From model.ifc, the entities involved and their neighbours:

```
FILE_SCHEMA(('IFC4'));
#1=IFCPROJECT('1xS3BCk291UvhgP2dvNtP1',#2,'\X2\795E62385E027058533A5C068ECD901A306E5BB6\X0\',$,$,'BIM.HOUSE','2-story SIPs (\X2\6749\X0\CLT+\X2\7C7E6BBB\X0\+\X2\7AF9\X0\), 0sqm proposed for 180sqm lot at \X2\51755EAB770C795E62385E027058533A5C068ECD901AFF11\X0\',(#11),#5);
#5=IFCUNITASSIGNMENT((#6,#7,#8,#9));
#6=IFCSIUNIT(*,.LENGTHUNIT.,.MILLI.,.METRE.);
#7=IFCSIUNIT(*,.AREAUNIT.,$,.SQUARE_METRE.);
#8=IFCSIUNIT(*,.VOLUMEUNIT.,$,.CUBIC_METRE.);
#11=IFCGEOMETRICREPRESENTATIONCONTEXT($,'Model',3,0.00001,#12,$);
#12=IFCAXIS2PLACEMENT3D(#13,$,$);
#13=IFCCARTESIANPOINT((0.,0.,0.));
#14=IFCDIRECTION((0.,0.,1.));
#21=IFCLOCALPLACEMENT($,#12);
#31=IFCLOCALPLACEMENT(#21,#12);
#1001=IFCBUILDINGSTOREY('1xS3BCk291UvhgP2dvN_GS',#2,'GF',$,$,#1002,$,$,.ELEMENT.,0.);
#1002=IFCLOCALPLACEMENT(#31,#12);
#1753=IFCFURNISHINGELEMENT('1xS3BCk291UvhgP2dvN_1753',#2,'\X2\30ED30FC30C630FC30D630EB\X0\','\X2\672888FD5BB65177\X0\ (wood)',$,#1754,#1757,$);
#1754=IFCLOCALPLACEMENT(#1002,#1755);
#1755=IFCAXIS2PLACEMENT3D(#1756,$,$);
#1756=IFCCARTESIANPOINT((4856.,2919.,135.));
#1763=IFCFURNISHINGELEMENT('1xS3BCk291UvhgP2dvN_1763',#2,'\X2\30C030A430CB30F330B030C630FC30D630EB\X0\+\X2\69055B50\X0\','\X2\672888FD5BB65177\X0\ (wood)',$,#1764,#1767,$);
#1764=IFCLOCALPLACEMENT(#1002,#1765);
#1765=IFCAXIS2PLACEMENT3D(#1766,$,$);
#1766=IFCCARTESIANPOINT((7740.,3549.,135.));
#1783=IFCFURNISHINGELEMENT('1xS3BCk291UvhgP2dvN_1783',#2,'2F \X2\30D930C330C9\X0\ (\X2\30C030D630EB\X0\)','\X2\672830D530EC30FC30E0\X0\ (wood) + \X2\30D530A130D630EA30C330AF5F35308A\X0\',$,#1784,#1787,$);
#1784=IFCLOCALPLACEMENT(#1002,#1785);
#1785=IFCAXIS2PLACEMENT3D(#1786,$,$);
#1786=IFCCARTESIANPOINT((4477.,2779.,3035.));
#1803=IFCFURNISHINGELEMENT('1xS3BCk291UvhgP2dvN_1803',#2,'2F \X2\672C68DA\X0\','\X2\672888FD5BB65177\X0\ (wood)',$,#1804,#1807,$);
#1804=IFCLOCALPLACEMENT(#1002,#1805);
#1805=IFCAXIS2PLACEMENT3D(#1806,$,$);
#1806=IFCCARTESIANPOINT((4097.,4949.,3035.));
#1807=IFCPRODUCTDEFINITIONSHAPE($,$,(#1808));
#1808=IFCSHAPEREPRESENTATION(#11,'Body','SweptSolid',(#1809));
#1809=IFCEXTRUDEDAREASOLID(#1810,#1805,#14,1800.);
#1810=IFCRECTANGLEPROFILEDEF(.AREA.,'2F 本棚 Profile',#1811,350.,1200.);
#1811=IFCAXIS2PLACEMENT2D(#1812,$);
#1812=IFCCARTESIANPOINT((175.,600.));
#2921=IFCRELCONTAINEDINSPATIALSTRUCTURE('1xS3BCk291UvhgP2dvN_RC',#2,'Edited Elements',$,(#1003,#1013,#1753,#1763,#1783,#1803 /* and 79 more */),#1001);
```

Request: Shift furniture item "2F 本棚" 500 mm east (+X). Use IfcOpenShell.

```python
import ifcopenshell
import ifcopenshell.api.geometry
import ifcopenshell.util.placement
import ifcopenshell.util.unit

model = ifcopenshell.open("model.ifc")
unit_scale = ifcopenshell.util.unit.calculate_unit_scale(model)

item = model.by_id(1803)
matrix = ifcopenshell.util.placement.get_local_placement(item.ObjectPlacement)
matrix[0, 3] += 0.5 / unit_scale
ifcopenshell.api.geometry.edit_object_placement(model, product=item, matrix=matrix, is_si=False)

print(ifcopenshell.util.placement.get_local_placement(item.ObjectPlacement).round(3) + 0.0)

model.write("model_rev.ifc")
```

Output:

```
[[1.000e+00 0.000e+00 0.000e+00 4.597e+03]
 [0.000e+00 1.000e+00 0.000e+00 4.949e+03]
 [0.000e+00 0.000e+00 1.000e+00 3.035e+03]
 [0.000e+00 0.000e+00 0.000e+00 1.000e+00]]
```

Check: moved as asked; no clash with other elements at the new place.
